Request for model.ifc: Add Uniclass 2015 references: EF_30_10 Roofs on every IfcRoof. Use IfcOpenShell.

First a look at what the model holds.

```python
import ifcopenshell

model = ifcopenshell.open("model.ifc")
print(model.schema)
print("classifications:", [c.Name for c in model.by_type("IfcClassification")])
for ifc_class in ("IfcDoor", "IfcRoof", "IfcStair", "IfcWall", "IfcWindow"):
    print(ifc_class, len(model.by_type(ifc_class)))
```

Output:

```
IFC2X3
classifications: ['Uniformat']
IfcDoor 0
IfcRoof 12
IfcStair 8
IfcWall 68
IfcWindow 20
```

```python
import ifcopenshell
import ifcopenshell.api.classification

model = ifcopenshell.open("model.ifc")

# IFC2X3 requires Source and Edition and has no link from the project to the system.
system = model.create_entity("IfcClassification", Source="NBS", Edition="2015", Name="Uniclass 2015")

codes = {
    "IfcRoof": ("EF_30_10", "Roofs"),
}
for ifc_class, (code, name) in codes.items():
    products = model.by_type(ifc_class)
    ifcopenshell.api.classification.add_reference(
        model, products=products, classification=system, identification=code, name=name
    )
    print(code, len(products))

model.write("model_updated.ifc")
```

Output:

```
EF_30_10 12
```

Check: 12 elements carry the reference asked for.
